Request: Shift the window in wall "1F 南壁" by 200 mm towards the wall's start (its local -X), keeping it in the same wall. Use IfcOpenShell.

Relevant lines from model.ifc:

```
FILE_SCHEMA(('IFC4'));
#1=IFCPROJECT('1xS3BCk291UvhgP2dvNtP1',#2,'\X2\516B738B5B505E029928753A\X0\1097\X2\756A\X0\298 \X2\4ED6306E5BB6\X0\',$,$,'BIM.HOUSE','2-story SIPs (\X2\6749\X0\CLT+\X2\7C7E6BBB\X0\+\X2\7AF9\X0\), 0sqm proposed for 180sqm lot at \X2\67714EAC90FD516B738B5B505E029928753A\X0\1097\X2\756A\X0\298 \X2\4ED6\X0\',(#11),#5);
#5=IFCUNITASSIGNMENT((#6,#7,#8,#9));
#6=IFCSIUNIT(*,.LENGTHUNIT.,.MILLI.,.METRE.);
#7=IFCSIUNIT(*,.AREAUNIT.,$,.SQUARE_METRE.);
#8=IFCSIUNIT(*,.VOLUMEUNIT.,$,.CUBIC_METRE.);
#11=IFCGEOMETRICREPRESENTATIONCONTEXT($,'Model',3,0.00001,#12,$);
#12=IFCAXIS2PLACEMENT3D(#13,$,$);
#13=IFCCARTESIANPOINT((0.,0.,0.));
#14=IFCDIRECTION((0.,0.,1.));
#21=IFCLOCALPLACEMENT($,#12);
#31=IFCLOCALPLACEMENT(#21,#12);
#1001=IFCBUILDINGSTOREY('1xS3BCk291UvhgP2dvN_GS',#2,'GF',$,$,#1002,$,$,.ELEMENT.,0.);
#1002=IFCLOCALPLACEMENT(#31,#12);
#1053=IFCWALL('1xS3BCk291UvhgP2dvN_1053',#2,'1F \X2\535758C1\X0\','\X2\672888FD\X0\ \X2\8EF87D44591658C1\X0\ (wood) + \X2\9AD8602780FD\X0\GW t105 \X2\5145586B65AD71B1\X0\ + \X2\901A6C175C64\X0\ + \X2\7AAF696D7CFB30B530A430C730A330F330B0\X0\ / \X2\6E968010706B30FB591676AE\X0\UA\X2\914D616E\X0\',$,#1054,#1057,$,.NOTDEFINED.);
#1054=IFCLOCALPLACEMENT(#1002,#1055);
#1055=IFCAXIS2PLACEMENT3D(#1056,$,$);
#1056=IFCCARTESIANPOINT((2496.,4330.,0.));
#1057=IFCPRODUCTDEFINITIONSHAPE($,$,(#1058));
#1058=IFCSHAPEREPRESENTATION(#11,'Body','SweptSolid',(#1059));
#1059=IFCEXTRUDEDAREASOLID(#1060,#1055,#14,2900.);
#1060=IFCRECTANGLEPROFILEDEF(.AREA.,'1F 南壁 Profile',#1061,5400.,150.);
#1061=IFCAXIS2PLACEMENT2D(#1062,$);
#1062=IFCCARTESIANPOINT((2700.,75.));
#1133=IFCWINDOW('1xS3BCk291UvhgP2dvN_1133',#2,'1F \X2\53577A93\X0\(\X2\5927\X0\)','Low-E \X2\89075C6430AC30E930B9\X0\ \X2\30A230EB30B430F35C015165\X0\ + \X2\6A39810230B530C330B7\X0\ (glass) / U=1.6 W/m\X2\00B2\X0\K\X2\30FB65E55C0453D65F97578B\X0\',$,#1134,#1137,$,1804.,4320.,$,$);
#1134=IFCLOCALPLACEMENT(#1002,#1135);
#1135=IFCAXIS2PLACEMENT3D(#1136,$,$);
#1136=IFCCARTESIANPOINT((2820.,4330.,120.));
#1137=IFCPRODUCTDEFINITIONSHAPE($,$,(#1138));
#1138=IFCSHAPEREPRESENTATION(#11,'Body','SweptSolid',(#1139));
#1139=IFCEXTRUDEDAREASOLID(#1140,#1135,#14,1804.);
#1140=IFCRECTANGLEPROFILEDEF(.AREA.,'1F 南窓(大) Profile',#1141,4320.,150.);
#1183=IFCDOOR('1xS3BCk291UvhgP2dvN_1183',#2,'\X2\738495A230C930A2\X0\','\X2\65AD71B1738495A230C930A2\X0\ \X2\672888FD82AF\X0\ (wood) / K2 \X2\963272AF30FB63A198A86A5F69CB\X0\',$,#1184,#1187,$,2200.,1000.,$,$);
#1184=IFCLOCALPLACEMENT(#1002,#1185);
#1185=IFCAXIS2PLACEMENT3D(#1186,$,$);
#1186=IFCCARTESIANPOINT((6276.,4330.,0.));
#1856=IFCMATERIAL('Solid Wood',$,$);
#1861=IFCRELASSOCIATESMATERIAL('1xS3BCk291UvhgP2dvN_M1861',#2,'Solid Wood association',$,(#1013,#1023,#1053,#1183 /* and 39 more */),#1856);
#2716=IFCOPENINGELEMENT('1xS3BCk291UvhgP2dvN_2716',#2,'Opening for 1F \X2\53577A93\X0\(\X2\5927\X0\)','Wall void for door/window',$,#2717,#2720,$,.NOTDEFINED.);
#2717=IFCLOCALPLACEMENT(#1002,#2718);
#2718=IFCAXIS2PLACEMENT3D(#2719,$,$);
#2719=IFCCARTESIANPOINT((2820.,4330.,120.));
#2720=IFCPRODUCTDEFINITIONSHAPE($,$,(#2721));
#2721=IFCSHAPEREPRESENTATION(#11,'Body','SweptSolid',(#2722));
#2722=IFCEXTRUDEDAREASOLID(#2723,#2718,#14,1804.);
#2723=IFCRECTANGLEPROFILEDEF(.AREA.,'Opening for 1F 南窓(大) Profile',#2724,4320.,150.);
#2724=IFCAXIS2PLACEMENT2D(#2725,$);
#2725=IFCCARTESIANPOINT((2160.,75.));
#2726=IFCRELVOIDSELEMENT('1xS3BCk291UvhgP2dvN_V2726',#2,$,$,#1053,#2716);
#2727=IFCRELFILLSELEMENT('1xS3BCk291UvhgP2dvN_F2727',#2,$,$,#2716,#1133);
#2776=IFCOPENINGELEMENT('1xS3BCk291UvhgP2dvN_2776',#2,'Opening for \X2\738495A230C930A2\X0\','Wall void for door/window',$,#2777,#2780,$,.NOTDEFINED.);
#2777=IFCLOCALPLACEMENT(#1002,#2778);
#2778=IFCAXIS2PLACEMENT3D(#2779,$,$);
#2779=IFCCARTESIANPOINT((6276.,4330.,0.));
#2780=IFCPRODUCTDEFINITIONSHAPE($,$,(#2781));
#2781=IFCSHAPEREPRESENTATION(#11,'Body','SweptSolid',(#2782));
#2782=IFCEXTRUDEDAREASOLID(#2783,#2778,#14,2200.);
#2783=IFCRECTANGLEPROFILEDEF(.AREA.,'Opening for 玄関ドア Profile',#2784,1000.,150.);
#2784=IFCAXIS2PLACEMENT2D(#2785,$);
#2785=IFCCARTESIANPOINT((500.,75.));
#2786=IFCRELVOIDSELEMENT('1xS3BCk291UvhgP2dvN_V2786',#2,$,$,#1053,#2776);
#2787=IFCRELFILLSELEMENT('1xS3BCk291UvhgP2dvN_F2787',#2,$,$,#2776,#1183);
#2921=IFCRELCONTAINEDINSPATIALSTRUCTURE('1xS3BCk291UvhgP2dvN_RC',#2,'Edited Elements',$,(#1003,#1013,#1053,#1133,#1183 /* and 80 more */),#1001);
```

```python
import ifcopenshell
import ifcopenshell.api.geometry
import ifcopenshell.util.placement

model = ifcopenshell.open("model.ifc")

window = model.by_guid("1xS3BCk291UvhgP2dvN_1133")
opening = window.FillsVoids[0].RelatingOpeningElement
wall = opening.VoidsElements[0].RelatingBuildingElement

wall_matrix = ifcopenshell.util.placement.get_local_placement(wall.ObjectPlacement)
shift = wall_matrix[:3, 0] * -200.0
before = ifcopenshell.util.placement.get_local_placement(window.ObjectPlacement)[:3, 3].copy()

# The window is not placed relative to its opening, so move both.
for product in (opening, window):
    matrix = ifcopenshell.util.placement.get_local_placement(product.ObjectPlacement)
    matrix[:3, 3] += shift
    ifcopenshell.api.geometry.edit_object_placement(model, product=product, matrix=matrix, is_si=False)

after = ifcopenshell.util.placement.get_local_placement(window.ObjectPlacement)[:3, 3]
print("window moved by", (after - before).round(3) + 0.0)

model.write("model_rev.ifc")
```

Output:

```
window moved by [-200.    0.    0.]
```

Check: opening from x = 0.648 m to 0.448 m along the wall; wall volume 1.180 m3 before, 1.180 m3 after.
